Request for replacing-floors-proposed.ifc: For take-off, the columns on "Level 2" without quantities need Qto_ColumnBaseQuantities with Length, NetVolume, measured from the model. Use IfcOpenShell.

First a look at what the model holds.

```python
import ifcopenshell
import ifcopenshell.util.element
import ifcopenshell.util.unit

model = ifcopenshell.open("replacing-floors-proposed.ifc")
print(model.schema)
for unit_type in ("LENGTHUNIT", "AREAUNIT", "VOLUMEUNIT"):
    print(unit_type, ifcopenshell.util.unit.calculate_unit_scale(model, unit_type))
storey = next(s for s in model.by_type("IfcBuildingStorey") if s.Name == "Level 2")
columns = [e for e in ifcopenshell.util.element.get_decomposition(storey) if e.is_a("IfcColumn")]
for e in sorted(columns, key=lambda e: e.id()):
    print(e.id(), e.is_a(), e.Name, list(ifcopenshell.util.element.get_psets(e, qtos_only=True)), sep=" | ")
```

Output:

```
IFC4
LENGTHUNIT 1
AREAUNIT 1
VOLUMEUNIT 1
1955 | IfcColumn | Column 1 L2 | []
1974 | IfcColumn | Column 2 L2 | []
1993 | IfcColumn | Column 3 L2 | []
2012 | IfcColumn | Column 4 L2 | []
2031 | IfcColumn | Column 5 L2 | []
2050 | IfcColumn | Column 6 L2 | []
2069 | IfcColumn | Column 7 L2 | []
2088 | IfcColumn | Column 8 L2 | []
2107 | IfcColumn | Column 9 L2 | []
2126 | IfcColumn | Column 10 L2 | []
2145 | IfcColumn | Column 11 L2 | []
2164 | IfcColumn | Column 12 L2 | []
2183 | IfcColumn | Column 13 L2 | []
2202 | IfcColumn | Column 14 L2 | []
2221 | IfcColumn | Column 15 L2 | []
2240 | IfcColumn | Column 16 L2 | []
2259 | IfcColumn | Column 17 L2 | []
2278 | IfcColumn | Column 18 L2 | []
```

```python
import ifcopenshell
import ifcopenshell.api.pset
import ifcopenshell.geom
import ifcopenshell.util.element
import ifcopenshell.util.shape
import ifcopenshell.util.unit

model = ifcopenshell.open("replacing-floors-proposed.ifc")
unit_scale = ifcopenshell.util.unit.calculate_unit_scale(model)
volume_scale = ifcopenshell.util.unit.calculate_unit_scale(model, "VOLUMEUNIT")
settings = ifcopenshell.geom.settings()

storey = next(s for s in model.by_type("IfcBuildingStorey") if s.Name == "Level 2")
columns = [e for e in ifcopenshell.util.element.get_decomposition(storey) if e.is_a("IfcColumn")]

for e in sorted(columns, key=lambda e: e.id()):
    if ifcopenshell.util.element.get_psets(e, qtos_only=True, should_inherit=False):
        continue
    # Geometry comes back in metres, in the element's own axes.
    shape = ifcopenshell.geom.create_shape(settings, e)
    values = {
        "Length": ifcopenshell.util.shape.get_z(shape.geometry) / unit_scale,
        "NetVolume": ifcopenshell.util.shape.get_volume(shape.geometry) / volume_scale,
    }
    qto = ifcopenshell.api.pset.add_qto(model, product=e, name="Qto_ColumnBaseQuantities")
    ifcopenshell.api.pset.edit_qto(model, qto=qto, properties=values)
    print(e.id(), {k: round(v, 3) for k, v in values.items()})

model.write("replacing-floors-proposed_rev.ifc")
```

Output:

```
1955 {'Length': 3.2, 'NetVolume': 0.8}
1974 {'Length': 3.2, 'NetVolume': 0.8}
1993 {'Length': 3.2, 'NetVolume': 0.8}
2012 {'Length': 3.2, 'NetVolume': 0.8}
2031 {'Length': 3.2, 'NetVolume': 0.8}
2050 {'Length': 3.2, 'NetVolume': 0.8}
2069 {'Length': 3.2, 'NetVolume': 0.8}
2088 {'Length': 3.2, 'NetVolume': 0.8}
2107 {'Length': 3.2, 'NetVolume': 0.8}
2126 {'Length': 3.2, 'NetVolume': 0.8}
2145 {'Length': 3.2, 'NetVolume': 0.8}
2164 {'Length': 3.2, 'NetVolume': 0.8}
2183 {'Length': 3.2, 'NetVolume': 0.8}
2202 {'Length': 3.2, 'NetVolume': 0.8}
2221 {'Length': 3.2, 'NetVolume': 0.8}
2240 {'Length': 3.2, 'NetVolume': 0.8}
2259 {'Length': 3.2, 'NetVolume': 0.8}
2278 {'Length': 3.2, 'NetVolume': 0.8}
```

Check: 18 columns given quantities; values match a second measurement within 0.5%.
